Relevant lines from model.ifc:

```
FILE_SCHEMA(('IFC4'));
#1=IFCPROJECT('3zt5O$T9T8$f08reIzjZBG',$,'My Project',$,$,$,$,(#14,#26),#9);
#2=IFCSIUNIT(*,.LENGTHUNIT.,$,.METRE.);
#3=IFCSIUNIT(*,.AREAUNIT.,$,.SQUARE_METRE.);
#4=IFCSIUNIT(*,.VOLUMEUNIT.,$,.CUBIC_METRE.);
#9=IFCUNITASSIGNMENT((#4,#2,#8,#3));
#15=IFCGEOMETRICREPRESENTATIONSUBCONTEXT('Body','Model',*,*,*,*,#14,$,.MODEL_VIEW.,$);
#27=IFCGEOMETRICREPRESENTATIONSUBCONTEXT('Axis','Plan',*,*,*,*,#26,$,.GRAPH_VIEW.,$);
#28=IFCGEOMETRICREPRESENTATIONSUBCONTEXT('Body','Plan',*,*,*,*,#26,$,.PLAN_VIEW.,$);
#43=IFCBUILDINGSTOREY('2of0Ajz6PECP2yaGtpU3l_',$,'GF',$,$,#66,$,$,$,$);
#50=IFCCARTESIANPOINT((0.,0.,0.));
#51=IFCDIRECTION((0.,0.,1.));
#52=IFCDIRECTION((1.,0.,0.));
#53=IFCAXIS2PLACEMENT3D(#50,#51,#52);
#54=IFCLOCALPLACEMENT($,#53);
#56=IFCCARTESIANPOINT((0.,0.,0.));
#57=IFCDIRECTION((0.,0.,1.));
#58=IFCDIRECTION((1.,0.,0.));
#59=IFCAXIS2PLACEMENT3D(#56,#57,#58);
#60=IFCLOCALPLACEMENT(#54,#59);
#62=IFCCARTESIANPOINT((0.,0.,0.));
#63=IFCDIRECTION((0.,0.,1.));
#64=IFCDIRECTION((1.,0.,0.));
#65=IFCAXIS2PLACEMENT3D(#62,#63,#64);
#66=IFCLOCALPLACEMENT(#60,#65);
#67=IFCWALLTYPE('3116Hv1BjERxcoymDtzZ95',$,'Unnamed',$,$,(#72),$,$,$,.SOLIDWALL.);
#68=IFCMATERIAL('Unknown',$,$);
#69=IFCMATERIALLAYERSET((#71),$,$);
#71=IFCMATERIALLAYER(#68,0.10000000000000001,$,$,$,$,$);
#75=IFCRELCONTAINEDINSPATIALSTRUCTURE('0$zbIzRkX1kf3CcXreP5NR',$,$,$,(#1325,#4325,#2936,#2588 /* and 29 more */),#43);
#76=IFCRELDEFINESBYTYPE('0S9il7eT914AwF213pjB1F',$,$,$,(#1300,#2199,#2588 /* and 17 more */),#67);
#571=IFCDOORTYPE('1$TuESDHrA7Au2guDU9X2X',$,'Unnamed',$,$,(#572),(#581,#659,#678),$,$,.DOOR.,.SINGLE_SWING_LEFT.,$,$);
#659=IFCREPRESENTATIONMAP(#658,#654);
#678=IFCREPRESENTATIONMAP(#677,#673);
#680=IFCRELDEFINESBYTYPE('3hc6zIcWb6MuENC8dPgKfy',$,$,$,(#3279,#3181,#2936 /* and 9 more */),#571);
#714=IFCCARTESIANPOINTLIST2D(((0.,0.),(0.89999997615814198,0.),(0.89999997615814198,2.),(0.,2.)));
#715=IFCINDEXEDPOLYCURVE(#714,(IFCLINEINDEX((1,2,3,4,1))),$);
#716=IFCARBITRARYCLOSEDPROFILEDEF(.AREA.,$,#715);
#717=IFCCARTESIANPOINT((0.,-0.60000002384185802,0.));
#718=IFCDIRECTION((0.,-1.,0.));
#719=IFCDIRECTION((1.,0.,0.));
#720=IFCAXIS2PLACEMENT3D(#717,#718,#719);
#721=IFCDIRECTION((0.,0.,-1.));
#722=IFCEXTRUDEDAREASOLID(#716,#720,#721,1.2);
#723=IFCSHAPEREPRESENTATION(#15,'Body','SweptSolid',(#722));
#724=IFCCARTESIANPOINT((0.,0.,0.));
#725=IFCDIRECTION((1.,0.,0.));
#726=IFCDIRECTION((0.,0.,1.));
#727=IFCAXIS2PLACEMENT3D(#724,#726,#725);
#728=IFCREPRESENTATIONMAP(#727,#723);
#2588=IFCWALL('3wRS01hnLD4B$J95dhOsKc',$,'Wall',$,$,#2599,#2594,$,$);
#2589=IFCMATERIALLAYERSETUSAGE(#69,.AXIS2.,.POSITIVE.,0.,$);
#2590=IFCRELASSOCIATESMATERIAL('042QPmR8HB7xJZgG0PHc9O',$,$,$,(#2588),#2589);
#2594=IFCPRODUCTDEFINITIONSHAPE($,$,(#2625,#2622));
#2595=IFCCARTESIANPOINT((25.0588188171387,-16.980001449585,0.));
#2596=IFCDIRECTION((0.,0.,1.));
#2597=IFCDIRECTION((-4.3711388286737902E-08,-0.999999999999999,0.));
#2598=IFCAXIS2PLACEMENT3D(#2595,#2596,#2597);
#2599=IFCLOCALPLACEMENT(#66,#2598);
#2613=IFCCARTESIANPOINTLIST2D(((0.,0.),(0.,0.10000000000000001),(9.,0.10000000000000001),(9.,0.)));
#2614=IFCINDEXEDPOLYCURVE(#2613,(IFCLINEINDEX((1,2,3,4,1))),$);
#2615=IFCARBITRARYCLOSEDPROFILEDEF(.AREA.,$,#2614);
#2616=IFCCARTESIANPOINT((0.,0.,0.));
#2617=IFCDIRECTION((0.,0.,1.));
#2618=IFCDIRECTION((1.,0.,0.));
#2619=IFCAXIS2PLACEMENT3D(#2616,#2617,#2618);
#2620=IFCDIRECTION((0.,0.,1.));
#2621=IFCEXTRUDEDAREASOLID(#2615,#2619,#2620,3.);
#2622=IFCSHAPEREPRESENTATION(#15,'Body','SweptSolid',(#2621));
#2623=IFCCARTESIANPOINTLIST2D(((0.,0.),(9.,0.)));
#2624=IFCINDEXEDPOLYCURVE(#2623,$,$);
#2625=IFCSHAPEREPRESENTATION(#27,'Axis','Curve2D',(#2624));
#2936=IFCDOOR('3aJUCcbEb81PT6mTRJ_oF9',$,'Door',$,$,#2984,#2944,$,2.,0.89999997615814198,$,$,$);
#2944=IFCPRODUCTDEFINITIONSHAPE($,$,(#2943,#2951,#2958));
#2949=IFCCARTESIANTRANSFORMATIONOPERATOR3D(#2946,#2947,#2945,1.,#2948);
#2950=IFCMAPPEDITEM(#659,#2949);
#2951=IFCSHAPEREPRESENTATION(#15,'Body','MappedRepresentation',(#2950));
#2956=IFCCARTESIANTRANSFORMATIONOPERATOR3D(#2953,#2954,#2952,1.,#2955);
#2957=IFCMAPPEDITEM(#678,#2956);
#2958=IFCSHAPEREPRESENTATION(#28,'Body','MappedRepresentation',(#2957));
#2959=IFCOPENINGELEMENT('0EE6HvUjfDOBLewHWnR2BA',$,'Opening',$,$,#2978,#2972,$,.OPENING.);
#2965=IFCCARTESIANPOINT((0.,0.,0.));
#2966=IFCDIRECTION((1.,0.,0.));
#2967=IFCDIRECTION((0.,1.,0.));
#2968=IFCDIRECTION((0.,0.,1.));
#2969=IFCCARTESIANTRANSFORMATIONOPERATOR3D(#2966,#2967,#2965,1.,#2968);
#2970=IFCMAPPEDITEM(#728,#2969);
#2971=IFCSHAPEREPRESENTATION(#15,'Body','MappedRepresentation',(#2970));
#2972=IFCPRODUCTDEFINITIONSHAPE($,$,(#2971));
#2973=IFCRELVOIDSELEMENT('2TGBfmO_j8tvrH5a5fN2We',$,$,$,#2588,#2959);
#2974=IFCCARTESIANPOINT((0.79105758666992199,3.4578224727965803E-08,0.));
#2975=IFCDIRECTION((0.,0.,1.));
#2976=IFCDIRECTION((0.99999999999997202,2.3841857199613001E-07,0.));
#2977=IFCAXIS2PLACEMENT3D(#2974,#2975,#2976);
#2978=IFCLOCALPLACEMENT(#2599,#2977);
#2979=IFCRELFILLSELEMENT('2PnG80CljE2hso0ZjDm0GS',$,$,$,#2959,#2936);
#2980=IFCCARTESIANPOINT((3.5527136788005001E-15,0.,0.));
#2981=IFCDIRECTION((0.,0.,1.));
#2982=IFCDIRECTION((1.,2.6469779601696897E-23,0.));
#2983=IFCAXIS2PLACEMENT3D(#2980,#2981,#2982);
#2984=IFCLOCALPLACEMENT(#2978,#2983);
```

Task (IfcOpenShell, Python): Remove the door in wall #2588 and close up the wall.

```python
import ifcopenshell
import ifcopenshell.api.feature
import ifcopenshell.api.root
import ifcopenshell.geom
import ifcopenshell.util.shape

model = ifcopenshell.open("model.ifc")
settings = ifcopenshell.geom.settings()


def volume(element):
    """Net volume in cubic metres, openings subtracted."""
    shape = ifcopenshell.geom.create_shape(settings, element)
    return ifcopenshell.util.shape.get_volume(shape.geometry)


door = model.by_guid("3aJUCcbEb81PT6mTRJ_oF9")
opening = door.FillsVoids[0].RelatingOpeningElement
wall = opening.VoidsElements[0].RelatingBuildingElement
before = volume(wall)

ifcopenshell.api.root.remove_product(model, product=door)
ifcopenshell.api.feature.remove_feature(model, feature=opening)

after = volume(wall)

print(f"wall volume {before:.3f} -> {after:.3f} m3")

model.write("model_updated.ifc")
```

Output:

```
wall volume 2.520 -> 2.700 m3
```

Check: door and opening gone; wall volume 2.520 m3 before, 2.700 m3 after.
